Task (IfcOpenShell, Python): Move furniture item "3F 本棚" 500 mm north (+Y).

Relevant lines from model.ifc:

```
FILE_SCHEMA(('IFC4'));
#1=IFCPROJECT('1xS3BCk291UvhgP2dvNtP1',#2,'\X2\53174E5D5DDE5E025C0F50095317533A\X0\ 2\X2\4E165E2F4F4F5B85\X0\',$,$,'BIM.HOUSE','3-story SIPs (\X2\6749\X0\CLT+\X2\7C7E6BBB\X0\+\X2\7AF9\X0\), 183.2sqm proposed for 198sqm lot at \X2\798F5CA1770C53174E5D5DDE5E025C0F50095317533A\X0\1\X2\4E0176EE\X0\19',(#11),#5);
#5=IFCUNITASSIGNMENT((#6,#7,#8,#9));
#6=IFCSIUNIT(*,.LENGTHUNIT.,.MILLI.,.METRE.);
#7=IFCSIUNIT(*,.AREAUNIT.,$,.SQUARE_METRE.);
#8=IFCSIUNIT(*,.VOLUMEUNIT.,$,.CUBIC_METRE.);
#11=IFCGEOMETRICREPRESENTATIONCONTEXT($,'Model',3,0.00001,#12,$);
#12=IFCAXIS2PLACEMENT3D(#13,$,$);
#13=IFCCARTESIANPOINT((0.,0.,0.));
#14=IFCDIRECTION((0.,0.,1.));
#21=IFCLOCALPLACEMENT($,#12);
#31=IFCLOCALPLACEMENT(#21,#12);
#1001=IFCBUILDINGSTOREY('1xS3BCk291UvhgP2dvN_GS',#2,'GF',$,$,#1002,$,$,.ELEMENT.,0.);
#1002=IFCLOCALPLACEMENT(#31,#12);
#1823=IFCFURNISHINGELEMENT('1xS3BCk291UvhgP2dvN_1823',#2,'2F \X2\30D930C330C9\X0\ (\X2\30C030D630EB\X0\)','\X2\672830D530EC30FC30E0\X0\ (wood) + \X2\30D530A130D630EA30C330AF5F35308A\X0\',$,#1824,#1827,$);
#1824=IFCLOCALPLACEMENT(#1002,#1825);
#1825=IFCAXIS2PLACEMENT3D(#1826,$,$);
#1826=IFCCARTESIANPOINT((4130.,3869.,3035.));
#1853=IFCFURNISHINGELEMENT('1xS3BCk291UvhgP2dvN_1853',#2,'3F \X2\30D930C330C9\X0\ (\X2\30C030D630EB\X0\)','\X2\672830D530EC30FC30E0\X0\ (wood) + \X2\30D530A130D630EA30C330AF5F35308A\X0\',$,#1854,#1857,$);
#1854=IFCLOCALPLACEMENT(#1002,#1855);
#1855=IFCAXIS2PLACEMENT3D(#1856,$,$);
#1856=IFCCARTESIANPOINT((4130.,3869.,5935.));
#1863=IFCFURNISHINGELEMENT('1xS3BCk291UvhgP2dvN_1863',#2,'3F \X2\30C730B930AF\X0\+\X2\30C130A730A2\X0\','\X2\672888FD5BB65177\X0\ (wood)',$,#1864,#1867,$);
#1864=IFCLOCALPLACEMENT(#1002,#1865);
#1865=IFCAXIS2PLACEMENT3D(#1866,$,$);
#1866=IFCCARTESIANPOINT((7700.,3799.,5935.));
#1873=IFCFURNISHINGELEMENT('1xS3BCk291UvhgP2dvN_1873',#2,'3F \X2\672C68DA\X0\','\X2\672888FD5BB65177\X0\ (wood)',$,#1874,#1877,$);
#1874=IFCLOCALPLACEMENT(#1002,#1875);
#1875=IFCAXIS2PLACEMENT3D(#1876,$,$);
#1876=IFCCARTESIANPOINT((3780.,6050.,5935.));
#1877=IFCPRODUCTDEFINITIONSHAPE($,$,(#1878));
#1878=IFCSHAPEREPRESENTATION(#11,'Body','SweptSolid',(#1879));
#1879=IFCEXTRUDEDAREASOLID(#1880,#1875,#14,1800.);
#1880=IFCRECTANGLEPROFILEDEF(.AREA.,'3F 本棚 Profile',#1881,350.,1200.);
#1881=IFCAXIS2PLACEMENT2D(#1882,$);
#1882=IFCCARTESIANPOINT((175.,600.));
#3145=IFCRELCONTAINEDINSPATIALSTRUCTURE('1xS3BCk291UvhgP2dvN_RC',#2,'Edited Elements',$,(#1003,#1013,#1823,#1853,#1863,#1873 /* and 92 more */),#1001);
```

```python
import ifcopenshell
import ifcopenshell.api.geometry
import ifcopenshell.util.placement

model = ifcopenshell.open("model.ifc")

item = model.by_guid("1xS3BCk291UvhgP2dvN_1873")
matrix = ifcopenshell.util.placement.get_local_placement(item.ObjectPlacement)
matrix[1, 3] += 500.0
ifcopenshell.api.geometry.edit_object_placement(model, product=item, matrix=matrix, is_si=False)

print(ifcopenshell.util.placement.get_local_placement(item.ObjectPlacement).round(3) + 0.0)

model.write("model-out.ifc")
```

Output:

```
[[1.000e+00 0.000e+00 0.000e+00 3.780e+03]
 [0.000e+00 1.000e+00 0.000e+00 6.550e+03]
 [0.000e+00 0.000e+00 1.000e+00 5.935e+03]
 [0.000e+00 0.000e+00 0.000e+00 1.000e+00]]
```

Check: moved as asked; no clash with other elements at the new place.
